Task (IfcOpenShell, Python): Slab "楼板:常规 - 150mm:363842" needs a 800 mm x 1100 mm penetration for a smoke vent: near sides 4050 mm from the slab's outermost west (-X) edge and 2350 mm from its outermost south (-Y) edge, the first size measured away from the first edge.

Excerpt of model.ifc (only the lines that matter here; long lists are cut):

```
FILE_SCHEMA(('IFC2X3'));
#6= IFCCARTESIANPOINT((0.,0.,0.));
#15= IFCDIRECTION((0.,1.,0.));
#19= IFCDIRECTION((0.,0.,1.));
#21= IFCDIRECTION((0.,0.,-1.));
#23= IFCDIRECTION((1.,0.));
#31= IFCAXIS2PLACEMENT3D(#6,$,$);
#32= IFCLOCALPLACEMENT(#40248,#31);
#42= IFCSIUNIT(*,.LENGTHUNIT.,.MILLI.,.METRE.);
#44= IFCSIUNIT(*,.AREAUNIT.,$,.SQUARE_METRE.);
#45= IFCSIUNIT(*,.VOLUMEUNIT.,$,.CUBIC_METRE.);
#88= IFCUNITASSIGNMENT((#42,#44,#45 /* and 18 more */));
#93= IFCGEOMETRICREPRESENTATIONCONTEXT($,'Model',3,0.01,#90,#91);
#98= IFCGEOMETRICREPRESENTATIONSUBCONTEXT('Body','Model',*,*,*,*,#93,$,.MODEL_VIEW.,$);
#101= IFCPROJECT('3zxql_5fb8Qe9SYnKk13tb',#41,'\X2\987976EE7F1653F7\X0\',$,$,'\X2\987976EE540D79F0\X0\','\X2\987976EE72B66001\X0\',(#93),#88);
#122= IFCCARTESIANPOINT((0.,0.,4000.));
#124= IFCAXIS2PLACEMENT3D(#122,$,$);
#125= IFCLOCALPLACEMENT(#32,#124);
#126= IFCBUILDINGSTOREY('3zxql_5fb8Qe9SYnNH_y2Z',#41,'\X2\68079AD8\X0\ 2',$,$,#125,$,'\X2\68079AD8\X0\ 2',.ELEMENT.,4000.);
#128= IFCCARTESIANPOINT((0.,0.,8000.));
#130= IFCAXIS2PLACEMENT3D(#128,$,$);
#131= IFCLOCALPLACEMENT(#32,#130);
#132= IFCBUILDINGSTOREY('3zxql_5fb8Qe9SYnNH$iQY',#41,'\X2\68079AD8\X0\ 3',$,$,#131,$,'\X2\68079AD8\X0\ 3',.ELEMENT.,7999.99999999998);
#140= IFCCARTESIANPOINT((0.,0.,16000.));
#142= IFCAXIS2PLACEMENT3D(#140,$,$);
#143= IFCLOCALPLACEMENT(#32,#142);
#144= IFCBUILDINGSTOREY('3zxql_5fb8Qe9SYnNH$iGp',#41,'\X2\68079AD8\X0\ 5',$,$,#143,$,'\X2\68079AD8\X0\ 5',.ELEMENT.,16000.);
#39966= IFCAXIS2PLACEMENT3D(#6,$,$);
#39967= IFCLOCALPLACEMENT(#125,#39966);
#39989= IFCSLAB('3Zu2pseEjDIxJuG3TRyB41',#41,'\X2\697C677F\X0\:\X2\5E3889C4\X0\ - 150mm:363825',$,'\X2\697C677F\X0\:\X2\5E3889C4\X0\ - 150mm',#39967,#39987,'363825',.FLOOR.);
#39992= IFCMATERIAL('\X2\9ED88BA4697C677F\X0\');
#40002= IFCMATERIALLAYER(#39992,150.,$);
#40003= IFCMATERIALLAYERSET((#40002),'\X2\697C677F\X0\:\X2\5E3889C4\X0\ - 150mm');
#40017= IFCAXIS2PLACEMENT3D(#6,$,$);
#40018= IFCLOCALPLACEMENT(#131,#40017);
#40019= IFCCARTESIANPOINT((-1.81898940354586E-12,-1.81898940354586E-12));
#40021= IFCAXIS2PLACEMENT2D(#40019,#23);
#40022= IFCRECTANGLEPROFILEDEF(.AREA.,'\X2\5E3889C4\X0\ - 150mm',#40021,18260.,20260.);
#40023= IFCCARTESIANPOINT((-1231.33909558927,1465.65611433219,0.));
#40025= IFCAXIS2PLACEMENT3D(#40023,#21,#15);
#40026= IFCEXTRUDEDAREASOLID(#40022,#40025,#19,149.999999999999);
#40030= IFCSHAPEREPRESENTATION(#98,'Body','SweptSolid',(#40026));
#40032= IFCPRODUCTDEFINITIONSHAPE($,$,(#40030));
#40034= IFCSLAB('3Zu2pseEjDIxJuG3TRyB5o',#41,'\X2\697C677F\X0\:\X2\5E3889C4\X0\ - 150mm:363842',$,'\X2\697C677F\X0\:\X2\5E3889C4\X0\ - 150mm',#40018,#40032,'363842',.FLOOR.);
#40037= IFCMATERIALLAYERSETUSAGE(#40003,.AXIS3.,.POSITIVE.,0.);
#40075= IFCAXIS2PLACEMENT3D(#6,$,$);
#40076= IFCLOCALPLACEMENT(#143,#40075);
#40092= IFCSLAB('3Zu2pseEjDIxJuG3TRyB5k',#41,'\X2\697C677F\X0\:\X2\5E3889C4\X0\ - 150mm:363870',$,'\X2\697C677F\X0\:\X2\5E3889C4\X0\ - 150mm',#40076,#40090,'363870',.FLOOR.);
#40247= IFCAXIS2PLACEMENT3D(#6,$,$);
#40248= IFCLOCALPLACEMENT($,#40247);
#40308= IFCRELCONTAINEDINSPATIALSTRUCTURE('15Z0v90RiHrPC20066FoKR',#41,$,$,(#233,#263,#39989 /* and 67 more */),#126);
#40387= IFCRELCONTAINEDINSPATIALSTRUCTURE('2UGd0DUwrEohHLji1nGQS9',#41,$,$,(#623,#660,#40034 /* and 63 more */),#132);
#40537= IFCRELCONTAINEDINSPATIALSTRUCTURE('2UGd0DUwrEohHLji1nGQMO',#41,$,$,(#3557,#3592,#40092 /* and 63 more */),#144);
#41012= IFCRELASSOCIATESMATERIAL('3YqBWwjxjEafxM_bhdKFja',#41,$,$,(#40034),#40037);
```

```python
import numpy as np
import ifcopenshell
import ifcopenshell.api.feature
import ifcopenshell.api.geometry
import ifcopenshell.api.root
import ifcopenshell.geom
import ifcopenshell.util.placement
import ifcopenshell.util.representation
import ifcopenshell.util.shape
import ifcopenshell.util.unit

model = ifcopenshell.open("model.ifc")
unit_scale = ifcopenshell.util.unit.calculate_unit_scale(model)
settings = ifcopenshell.geom.settings()


def volume(element):
    """Net volume in cubic metres, openings subtracted."""
    shape = ifcopenshell.geom.create_shape(settings, element)
    return ifcopenshell.util.shape.get_volume(shape.geometry)


slab = model.by_id(40034)
before = volume(slab)

# Extent in the slab's own axes, in metres. The edges named are its -X and -Y sides.
slab_shape = ifcopenshell.geom.create_shape(settings, slab)
vertices = ifcopenshell.util.shape.get_vertices(slab_shape.geometry)
x_min, y_min, bottom = vertices.min(axis=0)
top = vertices[:, 2].max()

opening = ifcopenshell.api.root.create_entity(model, ifc_class="IfcOpeningElement", name="Smoke vent opening")
context = ifcopenshell.util.representation.get_context(model, "Model", "Body", "MODEL_VIEW")
width, depth = 0.8, 1.1
outline = [(0.0, 0.0), (width, 0.0), (width, depth), (0.0, depth), (0.0, 0.0)]
# Overshoot both faces by 50 mm so the cut is clean.
shape = ifcopenshell.api.geometry.add_slab_representation(
    model, context=context, depth=top - bottom + 0.1, polyline=outline
)
ifcopenshell.api.geometry.assign_representation(model, product=opening, representation=shape)

matrix = ifcopenshell.util.placement.get_local_placement(slab.ObjectPlacement)
matrix[:, 3] = matrix @ np.append(np.array([x_min + 4.05, y_min + 2.35, bottom - 0.05]) / unit_scale, 1.0)
ifcopenshell.api.geometry.edit_object_placement(model, product=opening, matrix=matrix, is_si=False)
ifcopenshell.api.feature.add_feature(model, feature=opening, element=slab)

after = volume(slab)

print(f"slab volume {before:.3f} -> {after:.3f} m3")

model.write("model_v2.ifc")
```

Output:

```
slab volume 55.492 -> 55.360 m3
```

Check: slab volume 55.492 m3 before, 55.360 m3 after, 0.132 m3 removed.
